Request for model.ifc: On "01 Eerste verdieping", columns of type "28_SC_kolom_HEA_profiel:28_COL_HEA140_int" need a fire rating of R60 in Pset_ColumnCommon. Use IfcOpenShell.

First a look at what the model holds.

```python
import ifcopenshell
import ifcopenshell.util.element

model = ifcopenshell.open("model.ifc")
print(model.schema)
storey = next(s for s in model.by_type("IfcBuildingStorey") if s.Name == "01 Eerste verdieping")
columns = [e for e in ifcopenshell.util.element.get_decomposition(storey) if e.is_a("IfcColumn")]
seen = {}
for e in columns:
    element_type = ifcopenshell.util.element.get_type(e)
    key = (element_type.Name if element_type != e and element_type else None, ifcopenshell.util.element.get_pset(e, "Pset_ColumnCommon", "FireRating"))
    seen[key] = seen.get(key, 0) + 1
for (name, value), count in sorted(seen.items(), key=str):
    print(count, "x", name, "|", value)
```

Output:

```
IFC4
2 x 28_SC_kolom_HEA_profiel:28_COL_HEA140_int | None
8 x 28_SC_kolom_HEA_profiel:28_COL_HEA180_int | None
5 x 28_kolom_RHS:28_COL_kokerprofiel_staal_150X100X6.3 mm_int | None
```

```python
import ifcopenshell
import ifcopenshell.api.pset
import ifcopenshell.util.element

model = ifcopenshell.open("model.ifc")

storey = next(s for s in model.by_type("IfcBuildingStorey") if s.Name == "01 Eerste verdieping")
columns = [e for e in ifcopenshell.util.element.get_decomposition(storey) if e.is_a("IfcColumn")]

count = 0
for e in columns:
    element_type = ifcopenshell.util.element.get_type(e)
    if element_type in (None, e) or element_type.Name != "28_SC_kolom_HEA_profiel:28_COL_HEA140_int":
        continue
    # add_pset returns the element's existing set when there is one.
    pset = ifcopenshell.api.pset.add_pset(model, product=e, name="Pset_ColumnCommon")
    ifcopenshell.api.pset.edit_pset(model, pset=pset, properties={"FireRating": "R60"})
    count += 1

print(count, "columns updated")

model.write("model_updated.ifc")
```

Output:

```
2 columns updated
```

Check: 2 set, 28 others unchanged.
